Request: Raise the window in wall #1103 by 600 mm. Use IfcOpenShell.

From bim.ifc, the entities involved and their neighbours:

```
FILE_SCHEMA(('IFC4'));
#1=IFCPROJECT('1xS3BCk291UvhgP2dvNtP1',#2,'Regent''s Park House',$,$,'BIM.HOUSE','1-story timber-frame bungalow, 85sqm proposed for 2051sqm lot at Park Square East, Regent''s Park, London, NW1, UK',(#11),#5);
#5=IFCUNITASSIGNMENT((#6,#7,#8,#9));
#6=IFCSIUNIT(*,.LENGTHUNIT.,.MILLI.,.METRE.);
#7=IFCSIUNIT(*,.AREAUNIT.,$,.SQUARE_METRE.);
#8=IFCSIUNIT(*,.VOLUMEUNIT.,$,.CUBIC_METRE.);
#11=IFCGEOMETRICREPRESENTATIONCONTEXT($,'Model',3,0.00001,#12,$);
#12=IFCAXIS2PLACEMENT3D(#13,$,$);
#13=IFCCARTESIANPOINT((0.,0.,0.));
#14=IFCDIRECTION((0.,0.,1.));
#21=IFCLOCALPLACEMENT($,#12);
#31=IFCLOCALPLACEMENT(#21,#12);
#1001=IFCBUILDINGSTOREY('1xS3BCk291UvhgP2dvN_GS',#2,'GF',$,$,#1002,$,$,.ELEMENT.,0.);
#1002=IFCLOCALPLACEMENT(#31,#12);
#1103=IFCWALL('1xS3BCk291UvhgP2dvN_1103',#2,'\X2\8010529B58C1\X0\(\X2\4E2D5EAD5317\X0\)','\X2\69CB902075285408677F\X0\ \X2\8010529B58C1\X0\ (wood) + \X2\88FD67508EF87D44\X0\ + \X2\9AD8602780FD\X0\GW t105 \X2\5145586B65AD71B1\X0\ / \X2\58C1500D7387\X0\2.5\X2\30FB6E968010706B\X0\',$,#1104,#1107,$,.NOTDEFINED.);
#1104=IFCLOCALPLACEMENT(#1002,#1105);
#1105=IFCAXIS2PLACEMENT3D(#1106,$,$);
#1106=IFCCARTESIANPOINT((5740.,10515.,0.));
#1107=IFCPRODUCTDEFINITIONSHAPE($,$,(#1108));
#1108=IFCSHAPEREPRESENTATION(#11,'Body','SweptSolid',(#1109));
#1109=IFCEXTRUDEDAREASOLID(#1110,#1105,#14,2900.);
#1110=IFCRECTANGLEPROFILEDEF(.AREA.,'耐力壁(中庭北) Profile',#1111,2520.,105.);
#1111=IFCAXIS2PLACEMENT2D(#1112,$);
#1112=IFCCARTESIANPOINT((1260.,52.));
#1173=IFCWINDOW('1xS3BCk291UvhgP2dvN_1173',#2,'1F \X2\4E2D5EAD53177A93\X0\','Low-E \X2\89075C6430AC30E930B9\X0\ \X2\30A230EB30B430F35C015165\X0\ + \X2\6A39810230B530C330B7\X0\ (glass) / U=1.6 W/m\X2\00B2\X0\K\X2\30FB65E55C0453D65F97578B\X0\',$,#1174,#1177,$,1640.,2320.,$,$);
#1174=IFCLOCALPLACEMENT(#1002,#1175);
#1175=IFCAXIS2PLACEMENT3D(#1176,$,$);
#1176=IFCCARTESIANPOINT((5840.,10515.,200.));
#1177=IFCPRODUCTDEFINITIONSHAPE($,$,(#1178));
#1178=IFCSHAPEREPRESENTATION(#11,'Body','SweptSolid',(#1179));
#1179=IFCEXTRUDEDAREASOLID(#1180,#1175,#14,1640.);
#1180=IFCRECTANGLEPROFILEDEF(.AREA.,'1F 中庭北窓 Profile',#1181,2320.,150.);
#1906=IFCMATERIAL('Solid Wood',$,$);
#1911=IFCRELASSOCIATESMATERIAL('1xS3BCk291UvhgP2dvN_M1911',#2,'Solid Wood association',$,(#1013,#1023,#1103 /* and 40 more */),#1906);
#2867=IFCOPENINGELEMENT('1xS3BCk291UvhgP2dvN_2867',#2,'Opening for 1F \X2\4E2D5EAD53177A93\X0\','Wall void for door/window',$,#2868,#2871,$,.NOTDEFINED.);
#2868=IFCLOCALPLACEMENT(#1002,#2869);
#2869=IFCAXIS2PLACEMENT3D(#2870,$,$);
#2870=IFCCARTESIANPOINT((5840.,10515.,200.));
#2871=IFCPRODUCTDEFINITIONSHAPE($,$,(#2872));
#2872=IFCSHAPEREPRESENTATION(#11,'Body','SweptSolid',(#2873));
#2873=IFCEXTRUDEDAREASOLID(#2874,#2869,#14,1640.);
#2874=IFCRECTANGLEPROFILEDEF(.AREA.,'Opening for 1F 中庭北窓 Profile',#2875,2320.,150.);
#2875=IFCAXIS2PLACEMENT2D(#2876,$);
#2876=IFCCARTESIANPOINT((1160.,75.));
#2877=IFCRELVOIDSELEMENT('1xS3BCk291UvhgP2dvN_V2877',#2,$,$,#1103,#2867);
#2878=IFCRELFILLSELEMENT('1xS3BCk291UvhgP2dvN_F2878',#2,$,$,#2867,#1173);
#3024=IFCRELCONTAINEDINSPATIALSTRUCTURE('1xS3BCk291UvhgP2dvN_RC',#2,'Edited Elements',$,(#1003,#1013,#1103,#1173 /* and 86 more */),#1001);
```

```python
import numpy as np
import ifcopenshell
import ifcopenshell.api.geometry
import ifcopenshell.util.placement
import ifcopenshell.util.unit

model = ifcopenshell.open("bim.ifc")
unit_scale = ifcopenshell.util.unit.calculate_unit_scale(model)

window = model.by_id(1173)
opening = window.FillsVoids[0].RelatingOpeningElement
dz = 600.0

shift = np.array([0.0, 0.0, dz])
# The window is not placed relative to its opening, so move both.
for product in (opening, window):
    matrix = ifcopenshell.util.placement.get_local_placement(product.ObjectPlacement)
    matrix[:3, 3] += shift
    ifcopenshell.api.geometry.edit_object_placement(model, product=product, matrix=matrix, is_si=False)

print(f"moved by {dz * unit_scale:+.3f} m")

model.write("bim_edited.ifc")
```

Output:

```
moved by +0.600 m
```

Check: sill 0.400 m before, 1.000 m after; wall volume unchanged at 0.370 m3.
